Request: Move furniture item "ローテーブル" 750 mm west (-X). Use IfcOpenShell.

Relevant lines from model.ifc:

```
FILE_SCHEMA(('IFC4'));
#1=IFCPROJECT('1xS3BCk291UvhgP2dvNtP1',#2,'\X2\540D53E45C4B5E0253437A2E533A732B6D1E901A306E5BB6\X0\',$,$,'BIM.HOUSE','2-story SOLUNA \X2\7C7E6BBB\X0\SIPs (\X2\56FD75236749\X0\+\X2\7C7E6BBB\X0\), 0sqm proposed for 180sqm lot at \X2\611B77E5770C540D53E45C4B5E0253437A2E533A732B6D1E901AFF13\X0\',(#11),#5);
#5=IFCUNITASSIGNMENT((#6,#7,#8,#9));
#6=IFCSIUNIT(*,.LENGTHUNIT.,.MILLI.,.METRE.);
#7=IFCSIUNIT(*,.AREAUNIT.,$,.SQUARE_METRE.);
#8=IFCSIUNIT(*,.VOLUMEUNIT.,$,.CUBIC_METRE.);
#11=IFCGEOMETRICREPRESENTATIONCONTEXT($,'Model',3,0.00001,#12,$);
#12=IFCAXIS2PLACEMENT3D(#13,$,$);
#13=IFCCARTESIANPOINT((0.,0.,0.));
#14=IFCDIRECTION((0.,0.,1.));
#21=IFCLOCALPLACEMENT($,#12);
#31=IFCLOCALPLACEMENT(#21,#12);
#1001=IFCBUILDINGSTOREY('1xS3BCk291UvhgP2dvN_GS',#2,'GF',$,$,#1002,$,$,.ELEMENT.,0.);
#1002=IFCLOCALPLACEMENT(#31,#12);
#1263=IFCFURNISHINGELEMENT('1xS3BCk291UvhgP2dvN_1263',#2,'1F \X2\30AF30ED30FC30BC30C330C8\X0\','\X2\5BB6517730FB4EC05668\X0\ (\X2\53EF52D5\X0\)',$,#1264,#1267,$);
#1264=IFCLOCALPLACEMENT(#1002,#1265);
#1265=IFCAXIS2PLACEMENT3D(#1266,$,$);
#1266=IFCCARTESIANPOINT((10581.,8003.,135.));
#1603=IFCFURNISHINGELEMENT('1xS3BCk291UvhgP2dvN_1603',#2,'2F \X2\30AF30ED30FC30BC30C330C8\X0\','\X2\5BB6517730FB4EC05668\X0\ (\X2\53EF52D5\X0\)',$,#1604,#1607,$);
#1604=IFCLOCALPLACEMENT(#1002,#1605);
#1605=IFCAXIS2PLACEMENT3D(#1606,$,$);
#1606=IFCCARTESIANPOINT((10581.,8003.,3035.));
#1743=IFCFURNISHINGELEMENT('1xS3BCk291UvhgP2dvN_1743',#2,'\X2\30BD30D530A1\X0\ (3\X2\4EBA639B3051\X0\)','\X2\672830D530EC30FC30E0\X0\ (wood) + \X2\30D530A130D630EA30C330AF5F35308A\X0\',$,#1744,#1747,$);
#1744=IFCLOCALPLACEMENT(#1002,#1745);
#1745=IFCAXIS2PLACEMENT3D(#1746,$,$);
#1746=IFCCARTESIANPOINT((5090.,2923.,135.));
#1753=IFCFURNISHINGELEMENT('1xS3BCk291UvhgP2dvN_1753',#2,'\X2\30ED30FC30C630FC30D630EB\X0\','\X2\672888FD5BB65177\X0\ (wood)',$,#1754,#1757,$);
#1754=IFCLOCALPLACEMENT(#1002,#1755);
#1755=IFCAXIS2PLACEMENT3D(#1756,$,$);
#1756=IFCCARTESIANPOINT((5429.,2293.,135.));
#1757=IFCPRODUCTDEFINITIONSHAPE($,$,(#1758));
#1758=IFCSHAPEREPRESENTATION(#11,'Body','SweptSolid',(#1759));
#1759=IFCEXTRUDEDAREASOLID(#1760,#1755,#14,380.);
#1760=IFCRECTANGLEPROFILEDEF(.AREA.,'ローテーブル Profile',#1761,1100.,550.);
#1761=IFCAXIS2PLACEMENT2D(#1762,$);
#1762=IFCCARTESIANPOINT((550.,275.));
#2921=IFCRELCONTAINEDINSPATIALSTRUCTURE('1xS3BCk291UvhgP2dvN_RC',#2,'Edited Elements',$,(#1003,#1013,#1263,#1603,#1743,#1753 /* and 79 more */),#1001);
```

```python
import ifcopenshell
import ifcopenshell.api.geometry
import ifcopenshell.util.placement

model = ifcopenshell.open("model.ifc")

item = model.by_guid("1xS3BCk291UvhgP2dvN_1753")
matrix = ifcopenshell.util.placement.get_local_placement(item.ObjectPlacement)
matrix[0, 3] -= 750.0
ifcopenshell.api.geometry.edit_object_placement(model, product=item, matrix=matrix, is_si=False)

print(ifcopenshell.util.placement.get_local_placement(item.ObjectPlacement).round(3) + 0.0)

model.write("model_rev.ifc")
```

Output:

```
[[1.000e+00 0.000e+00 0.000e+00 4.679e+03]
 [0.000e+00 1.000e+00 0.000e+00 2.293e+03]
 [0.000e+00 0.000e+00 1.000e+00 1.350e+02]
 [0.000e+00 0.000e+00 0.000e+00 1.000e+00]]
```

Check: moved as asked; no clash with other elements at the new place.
